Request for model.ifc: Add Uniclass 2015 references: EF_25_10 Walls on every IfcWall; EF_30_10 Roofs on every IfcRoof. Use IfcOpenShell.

First a look at what the model holds.

```python
import ifcopenshell

model = ifcopenshell.open("model.ifc")
print(model.schema)
print("classifications:", [c.Name for c in model.by_type("IfcClassification")])
for ifc_class in ("IfcDoor", "IfcRoof", "IfcStair", "IfcWall", "IfcWindow"):
    print(ifc_class, len(model.by_type(ifc_class)))
```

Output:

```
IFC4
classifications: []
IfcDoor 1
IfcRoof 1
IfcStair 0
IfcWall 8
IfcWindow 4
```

```python
import ifcopenshell
import ifcopenshell.api.classification

model = ifcopenshell.open("model.ifc")

system = ifcopenshell.api.classification.add_classification(model, classification="Uniclass 2015")

codes = {
    "IfcWall": ("EF_25_10", "Walls"),
    "IfcRoof": ("EF_30_10", "Roofs"),
}
for ifc_class, (code, name) in codes.items():
    products = model.by_type(ifc_class)
    ifcopenshell.api.classification.add_reference(
        model, products=products, classification=system, identification=code, name=name
    )
    print(code, len(products))

model.write("model_updated.ifc")
```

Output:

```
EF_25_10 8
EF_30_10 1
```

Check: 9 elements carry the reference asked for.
